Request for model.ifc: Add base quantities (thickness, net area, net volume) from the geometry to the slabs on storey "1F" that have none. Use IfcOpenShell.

First a look at what the model holds.

```python
import ifcopenshell
import ifcopenshell.util.element
import ifcopenshell.util.unit

model = ifcopenshell.open("model.ifc")
print(model.schema)
for unit_type in ("LENGTHUNIT", "AREAUNIT", "VOLUMEUNIT"):
    print(unit_type, ifcopenshell.util.unit.calculate_unit_scale(model, unit_type))
storey = next(s for s in model.by_type("IfcBuildingStorey") if s.Name == "1F")
slabs = [e for e in ifcopenshell.util.element.get_decomposition(storey) if e.is_a("IfcSlab")]
for e in sorted(slabs, key=lambda e: e.id()):
    print(e.id(), e.is_a(), e.Name, list(ifcopenshell.util.element.get_psets(e, qtos_only=True)), sep=" | ")
```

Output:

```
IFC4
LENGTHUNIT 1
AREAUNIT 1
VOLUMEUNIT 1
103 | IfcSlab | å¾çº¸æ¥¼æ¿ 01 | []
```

```python
import ifcopenshell
import ifcopenshell.api.pset
import ifcopenshell.geom
import ifcopenshell.util.element
import ifcopenshell.util.shape
import ifcopenshell.util.unit

model = ifcopenshell.open("model.ifc")
unit_scale = ifcopenshell.util.unit.calculate_unit_scale(model)
area_scale = ifcopenshell.util.unit.calculate_unit_scale(model, "AREAUNIT")
volume_scale = ifcopenshell.util.unit.calculate_unit_scale(model, "VOLUMEUNIT")
settings = ifcopenshell.geom.settings()

storey = next(s for s in model.by_type("IfcBuildingStorey") if s.Name == "1F")
slabs = [e for e in ifcopenshell.util.element.get_decomposition(storey) if e.is_a("IfcSlab")]

for e in sorted(slabs, key=lambda e: e.id()):
    if ifcopenshell.util.element.get_psets(e, qtos_only=True, should_inherit=False):
        continue
    # Geometry comes back in metres, in the element's own axes.
    shape = ifcopenshell.geom.create_shape(settings, e)
    values = {
        "Width": ifcopenshell.util.shape.get_z(shape.geometry) / unit_scale,
        "NetArea": ifcopenshell.util.shape.get_footprint_area(shape.geometry) / area_scale,
        "NetVolume": ifcopenshell.util.shape.get_volume(shape.geometry) / volume_scale,
    }
    qto = ifcopenshell.api.pset.add_qto(model, product=e, name="Qto_SlabBaseQuantities")
    ifcopenshell.api.pset.edit_qto(model, qto=qto, properties=values)
    print(e.id(), {k: round(v, 3) for k, v in values.items()})

model.write("model_v2.ifc")
```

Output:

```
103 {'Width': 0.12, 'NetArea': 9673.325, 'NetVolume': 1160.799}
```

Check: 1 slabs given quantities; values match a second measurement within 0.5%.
